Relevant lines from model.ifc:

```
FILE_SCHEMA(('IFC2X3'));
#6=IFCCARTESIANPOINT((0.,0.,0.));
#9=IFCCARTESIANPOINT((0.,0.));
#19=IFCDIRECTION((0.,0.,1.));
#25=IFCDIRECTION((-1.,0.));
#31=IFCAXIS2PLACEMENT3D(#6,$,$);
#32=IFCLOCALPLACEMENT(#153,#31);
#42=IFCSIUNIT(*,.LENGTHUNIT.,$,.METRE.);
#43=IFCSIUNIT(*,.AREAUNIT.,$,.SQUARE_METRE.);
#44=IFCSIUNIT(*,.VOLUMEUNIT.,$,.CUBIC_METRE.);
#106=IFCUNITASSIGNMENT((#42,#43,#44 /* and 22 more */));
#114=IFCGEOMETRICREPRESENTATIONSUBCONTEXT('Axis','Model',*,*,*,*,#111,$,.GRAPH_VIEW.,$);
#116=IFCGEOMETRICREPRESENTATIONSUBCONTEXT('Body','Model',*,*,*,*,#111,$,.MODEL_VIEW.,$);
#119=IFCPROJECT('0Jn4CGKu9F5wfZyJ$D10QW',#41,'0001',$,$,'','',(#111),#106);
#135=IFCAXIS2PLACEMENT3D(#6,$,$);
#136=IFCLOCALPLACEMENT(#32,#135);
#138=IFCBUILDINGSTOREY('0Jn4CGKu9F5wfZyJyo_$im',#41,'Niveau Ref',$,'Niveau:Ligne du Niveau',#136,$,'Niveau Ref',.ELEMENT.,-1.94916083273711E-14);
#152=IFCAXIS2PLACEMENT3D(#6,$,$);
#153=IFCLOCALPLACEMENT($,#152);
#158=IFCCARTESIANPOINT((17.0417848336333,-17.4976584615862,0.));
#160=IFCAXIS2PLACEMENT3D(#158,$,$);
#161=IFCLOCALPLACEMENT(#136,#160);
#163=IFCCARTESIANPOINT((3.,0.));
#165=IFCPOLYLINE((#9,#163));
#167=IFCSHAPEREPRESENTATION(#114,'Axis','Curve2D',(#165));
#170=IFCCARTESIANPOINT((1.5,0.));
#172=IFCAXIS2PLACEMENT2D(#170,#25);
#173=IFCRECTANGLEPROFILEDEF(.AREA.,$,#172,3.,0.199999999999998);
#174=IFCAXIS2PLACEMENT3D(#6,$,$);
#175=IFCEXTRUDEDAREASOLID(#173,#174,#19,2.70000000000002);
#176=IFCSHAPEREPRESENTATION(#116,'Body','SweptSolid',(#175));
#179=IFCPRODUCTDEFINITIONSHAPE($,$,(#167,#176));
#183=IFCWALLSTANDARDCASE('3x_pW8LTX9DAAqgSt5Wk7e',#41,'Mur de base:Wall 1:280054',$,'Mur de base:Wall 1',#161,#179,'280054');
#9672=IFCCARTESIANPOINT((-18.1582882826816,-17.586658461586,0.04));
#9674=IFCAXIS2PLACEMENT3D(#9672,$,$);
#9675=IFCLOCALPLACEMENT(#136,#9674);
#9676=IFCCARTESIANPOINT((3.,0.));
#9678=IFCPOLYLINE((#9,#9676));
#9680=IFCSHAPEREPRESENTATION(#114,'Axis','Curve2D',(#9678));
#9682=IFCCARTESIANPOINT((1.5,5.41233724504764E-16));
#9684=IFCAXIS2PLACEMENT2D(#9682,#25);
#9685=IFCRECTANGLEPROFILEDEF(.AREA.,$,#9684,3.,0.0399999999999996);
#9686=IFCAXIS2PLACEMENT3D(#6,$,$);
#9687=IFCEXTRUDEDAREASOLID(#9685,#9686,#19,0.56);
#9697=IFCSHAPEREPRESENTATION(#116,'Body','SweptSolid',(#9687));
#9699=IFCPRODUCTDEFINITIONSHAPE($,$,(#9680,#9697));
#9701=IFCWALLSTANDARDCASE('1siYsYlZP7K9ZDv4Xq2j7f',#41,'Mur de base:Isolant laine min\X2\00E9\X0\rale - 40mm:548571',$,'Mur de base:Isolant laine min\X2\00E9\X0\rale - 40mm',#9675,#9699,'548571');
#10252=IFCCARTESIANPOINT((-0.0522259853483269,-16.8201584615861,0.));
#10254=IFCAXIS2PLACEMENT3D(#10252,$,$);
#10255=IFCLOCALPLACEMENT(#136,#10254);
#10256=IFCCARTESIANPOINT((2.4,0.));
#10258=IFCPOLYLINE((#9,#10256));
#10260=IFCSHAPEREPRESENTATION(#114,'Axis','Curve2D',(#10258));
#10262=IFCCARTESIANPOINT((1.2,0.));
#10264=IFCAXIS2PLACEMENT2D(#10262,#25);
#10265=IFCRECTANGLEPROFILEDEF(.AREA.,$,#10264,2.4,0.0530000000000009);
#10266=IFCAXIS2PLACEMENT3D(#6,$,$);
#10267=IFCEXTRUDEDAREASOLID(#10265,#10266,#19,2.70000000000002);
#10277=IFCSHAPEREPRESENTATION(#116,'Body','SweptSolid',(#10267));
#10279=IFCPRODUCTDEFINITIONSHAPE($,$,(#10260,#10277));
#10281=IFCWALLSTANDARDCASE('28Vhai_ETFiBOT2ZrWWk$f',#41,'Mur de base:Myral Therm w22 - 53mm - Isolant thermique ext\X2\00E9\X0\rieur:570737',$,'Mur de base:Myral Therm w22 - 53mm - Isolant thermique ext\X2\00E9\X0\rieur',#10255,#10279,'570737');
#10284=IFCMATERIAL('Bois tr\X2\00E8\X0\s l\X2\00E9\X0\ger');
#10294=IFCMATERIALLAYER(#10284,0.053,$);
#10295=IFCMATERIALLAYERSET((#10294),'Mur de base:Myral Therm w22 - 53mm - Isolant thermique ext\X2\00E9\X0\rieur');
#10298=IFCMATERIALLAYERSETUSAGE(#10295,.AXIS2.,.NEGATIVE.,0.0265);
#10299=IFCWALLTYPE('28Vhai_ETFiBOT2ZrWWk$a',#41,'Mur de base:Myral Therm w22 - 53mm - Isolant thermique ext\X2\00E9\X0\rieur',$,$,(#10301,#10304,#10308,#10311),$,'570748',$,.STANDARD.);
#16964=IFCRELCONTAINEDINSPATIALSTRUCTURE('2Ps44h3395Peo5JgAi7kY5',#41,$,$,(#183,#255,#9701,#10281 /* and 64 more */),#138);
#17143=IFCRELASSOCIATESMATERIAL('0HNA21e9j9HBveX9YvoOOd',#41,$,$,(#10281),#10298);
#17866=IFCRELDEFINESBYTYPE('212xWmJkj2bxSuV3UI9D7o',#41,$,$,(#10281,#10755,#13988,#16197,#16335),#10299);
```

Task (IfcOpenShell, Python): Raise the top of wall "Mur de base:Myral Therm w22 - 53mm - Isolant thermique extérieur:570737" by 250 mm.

```python
import ifcopenshell
import ifcopenshell.geom
import ifcopenshell.util.representation
import ifcopenshell.util.shape
import ifcopenshell.util.unit

model = ifcopenshell.open("model.ifc")
unit_scale = ifcopenshell.util.unit.calculate_unit_scale(model)
settings = ifcopenshell.geom.settings()


def volume(element):
    """Net volume in cubic metres, openings subtracted."""
    shape = ifcopenshell.geom.create_shape(settings, element)
    return ifcopenshell.util.shape.get_volume(shape.geometry)


wall = model.by_guid("28Vhai_ETFiBOT2ZrWWk$f")
before = volume(wall)

body = ifcopenshell.util.representation.get_representation(wall, "Model", "Body")
solid = body.Items[0]
old_height = solid.Depth
solid.Depth += 0.25 / unit_scale
after = volume(wall)

print(f"height {old_height:g} -> {solid.Depth:g}, volume {before:.3f} -> {after:.3f} m3")

model.write("model_v2.ifc")
```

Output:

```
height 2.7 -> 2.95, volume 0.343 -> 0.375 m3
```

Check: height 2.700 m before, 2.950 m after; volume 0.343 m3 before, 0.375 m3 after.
